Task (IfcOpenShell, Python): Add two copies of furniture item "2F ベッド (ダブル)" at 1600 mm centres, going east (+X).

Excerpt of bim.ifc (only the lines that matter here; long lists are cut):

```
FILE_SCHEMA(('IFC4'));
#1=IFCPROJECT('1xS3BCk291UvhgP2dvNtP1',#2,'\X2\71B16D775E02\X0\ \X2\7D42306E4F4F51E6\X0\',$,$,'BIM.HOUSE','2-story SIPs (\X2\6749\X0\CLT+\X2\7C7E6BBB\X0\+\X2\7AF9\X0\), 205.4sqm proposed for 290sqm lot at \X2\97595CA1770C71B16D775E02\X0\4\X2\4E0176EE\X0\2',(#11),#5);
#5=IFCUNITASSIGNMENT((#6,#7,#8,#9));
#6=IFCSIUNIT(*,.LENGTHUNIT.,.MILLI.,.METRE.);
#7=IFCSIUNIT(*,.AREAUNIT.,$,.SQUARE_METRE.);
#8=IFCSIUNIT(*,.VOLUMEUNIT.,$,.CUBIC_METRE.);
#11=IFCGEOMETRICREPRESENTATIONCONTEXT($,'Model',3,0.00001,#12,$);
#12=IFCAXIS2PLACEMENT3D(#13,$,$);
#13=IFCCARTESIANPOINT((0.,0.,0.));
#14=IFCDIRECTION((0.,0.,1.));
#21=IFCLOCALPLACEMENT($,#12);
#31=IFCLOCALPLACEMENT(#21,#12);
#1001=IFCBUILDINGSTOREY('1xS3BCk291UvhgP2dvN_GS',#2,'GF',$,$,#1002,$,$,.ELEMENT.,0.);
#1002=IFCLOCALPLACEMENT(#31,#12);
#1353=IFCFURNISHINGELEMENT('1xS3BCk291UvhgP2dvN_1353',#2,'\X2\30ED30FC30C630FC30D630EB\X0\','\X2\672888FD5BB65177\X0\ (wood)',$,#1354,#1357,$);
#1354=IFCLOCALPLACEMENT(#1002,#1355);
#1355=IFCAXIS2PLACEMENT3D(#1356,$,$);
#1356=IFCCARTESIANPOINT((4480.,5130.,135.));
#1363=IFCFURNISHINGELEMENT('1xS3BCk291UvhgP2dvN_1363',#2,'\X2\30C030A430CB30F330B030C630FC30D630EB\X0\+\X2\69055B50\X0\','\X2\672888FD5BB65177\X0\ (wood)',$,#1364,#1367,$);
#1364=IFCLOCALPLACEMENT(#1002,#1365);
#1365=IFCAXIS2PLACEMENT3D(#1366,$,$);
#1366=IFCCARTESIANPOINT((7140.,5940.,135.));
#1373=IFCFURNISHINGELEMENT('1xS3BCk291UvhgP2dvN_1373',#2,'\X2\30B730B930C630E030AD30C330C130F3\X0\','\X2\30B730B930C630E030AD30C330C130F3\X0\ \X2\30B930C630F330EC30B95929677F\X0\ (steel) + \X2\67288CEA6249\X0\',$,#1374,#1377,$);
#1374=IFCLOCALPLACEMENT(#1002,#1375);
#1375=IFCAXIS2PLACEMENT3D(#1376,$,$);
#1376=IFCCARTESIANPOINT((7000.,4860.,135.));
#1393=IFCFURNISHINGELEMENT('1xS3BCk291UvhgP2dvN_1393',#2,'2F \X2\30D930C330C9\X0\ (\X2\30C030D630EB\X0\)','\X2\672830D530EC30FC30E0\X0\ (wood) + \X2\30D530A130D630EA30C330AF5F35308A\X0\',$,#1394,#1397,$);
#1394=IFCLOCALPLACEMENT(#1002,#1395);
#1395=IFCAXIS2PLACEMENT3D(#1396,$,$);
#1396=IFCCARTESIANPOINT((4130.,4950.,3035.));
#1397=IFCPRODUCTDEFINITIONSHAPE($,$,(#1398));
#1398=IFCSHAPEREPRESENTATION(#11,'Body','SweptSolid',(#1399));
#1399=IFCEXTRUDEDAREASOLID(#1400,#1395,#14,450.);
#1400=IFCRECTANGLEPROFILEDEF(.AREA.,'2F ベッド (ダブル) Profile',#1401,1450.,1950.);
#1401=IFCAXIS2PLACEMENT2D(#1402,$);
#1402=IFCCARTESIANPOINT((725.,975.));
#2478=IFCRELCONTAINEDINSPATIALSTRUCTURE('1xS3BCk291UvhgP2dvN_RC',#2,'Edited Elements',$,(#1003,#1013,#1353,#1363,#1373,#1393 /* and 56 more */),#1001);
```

```python
import numpy as np
import ifcopenshell
import ifcopenshell.api.geometry
import ifcopenshell.api.root
import ifcopenshell.util.element
import ifcopenshell.util.placement

model = ifcopenshell.open("bim.ifc")


def reuse_history(source, copy):
    """copy_class also copies each property set's owner history, people and application; keep the originals."""
    for rel in copy.IsDefinedBy:
        if rel.is_a("IfcRelDefinesByProperties") and (history := rel.RelatingPropertyDefinition.OwnerHistory):
            rel.RelatingPropertyDefinition.OwnerHistory = source.OwnerHistory
            ifcopenshell.util.element.remove_deep2(model, history)


source = model.by_guid("1xS3BCk291UvhgP2dvN_1393")
base = ifcopenshell.util.placement.get_local_placement(source.ObjectPlacement)
step = np.array([1.0, 0.0, 0.0]) * 1600.0

for i in range(1, 3):
    copy = ifcopenshell.api.root.copy_class(model, product=source)
    copy.Representation = ifcopenshell.util.element.copy_deep(
        model, source.Representation, exclude=["IfcGeometricRepresentationContext", "IfcRepresentationMap"]
    )
    reuse_history(source, copy)
    matrix = base.copy()
    matrix[:3, 3] += i * step
    print("added at", matrix[:3, 3].round(3) + 0.0)
    ifcopenshell.api.geometry.edit_object_placement(model, product=copy, matrix=matrix, is_si=False)

model.write("bim_updated.ifc")
```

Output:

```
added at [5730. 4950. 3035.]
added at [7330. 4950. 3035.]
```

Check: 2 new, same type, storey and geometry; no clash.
